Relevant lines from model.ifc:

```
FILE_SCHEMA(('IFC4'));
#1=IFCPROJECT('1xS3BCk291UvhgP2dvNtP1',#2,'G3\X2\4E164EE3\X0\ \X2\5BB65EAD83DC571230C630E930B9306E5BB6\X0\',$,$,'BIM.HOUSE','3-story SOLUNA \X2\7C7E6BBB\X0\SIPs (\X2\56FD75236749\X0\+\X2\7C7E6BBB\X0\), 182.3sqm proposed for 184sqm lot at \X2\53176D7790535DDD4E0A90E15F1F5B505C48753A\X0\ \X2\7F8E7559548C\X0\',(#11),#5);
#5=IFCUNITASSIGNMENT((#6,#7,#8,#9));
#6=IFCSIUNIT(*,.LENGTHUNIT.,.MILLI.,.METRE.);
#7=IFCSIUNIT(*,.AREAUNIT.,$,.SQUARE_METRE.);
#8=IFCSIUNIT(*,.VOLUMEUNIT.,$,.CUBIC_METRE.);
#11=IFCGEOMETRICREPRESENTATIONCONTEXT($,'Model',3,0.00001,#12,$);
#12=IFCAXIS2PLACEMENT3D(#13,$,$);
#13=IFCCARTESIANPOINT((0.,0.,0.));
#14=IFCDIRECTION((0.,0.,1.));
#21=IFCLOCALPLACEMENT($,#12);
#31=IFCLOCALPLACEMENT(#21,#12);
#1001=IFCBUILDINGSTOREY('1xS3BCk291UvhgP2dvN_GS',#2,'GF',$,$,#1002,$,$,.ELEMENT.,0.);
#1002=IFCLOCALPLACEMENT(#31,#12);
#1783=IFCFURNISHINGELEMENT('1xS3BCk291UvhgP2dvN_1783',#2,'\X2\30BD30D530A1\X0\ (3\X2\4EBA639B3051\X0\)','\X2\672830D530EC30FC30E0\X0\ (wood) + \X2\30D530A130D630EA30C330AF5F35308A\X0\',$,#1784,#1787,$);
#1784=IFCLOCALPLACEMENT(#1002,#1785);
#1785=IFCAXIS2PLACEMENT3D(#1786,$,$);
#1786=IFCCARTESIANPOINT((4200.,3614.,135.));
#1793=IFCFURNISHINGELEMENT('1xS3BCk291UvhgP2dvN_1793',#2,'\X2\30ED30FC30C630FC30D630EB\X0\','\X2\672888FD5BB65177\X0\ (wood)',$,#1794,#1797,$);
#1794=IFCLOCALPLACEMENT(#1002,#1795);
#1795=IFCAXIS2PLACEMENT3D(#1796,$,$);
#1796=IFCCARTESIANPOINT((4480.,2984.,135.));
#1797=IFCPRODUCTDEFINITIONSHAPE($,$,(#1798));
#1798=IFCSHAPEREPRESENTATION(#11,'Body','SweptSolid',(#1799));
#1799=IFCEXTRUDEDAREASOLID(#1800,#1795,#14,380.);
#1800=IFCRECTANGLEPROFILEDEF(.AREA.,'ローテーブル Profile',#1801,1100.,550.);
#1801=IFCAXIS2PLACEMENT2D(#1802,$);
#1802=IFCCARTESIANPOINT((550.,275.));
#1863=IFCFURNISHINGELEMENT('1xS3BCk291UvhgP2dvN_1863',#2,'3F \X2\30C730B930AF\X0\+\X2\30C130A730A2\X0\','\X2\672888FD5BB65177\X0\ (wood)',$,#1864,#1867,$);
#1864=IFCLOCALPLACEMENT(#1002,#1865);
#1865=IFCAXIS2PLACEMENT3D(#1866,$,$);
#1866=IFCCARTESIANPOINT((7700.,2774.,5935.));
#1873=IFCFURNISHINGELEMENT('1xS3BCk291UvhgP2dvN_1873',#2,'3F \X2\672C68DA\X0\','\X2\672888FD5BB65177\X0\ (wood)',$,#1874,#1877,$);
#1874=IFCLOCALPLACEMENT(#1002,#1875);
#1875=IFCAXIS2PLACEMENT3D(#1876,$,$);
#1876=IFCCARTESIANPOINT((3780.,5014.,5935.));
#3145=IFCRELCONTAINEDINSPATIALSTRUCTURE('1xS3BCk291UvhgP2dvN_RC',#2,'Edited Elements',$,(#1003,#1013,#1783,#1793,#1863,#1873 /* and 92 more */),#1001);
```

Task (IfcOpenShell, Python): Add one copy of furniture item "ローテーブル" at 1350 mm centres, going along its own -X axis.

```python
import ifcopenshell
import ifcopenshell.api.geometry
import ifcopenshell.api.root
import ifcopenshell.util.element
import ifcopenshell.util.placement
import ifcopenshell.util.unit

model = ifcopenshell.open("model.ifc")
unit_scale = ifcopenshell.util.unit.calculate_unit_scale(model)


def reuse_history(source, copy):
    """copy_class also copies each property set's owner history, people and application; keep the originals."""
    for rel in copy.IsDefinedBy:
        if rel.is_a("IfcRelDefinesByProperties") and (history := rel.RelatingPropertyDefinition.OwnerHistory):
            rel.RelatingPropertyDefinition.OwnerHistory = source.OwnerHistory
            ifcopenshell.util.element.remove_deep2(model, history)


source = model.by_guid("1xS3BCk291UvhgP2dvN_1793")
base = ifcopenshell.util.placement.get_local_placement(source.ObjectPlacement)
step = -base[:3, 0] * 1.35 / unit_scale

for i in range(1, 2):
    copy = ifcopenshell.api.root.copy_class(model, product=source)
    copy.Representation = ifcopenshell.util.element.copy_deep(
        model, source.Representation, exclude=["IfcGeometricRepresentationContext", "IfcRepresentationMap"]
    )
    reuse_history(source, copy)
    matrix = base.copy()
    matrix[:3, 3] += i * step
    print("added at", matrix[:3, 3].round(3) + 0.0)
    ifcopenshell.api.geometry.edit_object_placement(model, product=copy, matrix=matrix, is_si=False)

model.write("model_v2.ifc")
```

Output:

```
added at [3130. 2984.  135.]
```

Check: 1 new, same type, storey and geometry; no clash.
